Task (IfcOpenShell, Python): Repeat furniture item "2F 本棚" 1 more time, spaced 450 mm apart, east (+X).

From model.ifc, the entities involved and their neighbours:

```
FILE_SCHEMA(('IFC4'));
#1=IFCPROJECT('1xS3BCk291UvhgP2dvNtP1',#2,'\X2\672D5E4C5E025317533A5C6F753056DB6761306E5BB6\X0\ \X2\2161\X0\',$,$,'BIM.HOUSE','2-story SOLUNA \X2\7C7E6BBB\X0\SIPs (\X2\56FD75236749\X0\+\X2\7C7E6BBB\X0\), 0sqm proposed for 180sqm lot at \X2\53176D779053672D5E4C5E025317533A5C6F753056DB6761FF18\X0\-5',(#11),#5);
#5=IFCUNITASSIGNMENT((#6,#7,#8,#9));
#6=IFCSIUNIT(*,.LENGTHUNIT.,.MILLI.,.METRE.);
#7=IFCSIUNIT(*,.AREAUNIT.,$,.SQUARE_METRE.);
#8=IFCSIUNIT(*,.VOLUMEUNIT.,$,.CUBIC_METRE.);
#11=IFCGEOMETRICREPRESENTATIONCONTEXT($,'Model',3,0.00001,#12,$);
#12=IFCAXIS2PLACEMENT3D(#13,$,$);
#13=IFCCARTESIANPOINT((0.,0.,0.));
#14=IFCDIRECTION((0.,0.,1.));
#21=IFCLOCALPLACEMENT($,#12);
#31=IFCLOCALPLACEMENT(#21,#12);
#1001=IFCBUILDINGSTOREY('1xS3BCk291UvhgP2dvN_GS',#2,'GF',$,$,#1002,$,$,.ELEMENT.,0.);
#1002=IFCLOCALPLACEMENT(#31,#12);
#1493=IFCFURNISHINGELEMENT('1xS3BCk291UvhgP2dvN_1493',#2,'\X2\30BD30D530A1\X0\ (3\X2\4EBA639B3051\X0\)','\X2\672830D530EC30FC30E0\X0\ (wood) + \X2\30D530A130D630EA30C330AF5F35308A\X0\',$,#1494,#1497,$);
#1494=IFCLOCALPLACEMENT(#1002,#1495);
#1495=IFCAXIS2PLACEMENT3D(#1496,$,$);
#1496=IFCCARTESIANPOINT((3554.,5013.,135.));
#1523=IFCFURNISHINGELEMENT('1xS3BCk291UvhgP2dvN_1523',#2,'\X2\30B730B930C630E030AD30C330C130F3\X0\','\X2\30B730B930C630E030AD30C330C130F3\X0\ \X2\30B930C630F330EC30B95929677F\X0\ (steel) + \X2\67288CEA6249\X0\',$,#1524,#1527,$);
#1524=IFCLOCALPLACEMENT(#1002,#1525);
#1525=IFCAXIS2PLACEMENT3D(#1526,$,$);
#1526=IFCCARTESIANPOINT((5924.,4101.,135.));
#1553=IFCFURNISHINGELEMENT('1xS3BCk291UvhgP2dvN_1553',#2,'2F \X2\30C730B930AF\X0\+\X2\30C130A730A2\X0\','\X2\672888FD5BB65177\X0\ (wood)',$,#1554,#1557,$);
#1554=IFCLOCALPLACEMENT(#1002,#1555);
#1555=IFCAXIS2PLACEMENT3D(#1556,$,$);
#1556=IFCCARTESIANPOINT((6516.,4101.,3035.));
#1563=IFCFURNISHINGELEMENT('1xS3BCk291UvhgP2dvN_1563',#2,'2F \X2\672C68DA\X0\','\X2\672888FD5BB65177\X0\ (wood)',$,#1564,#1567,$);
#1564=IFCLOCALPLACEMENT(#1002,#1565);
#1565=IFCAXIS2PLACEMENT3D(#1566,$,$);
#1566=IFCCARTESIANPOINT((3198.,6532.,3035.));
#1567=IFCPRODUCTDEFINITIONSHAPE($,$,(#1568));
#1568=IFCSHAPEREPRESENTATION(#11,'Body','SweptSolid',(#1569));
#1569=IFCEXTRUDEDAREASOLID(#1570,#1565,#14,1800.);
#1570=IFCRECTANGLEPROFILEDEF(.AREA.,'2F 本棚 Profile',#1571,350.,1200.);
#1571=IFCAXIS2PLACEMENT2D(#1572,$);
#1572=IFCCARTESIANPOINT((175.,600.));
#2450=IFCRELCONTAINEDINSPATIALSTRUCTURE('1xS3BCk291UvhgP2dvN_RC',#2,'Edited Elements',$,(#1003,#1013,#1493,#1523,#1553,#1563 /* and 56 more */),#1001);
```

```python
import numpy as np
import ifcopenshell
import ifcopenshell.api.geometry
import ifcopenshell.api.root
import ifcopenshell.util.element
import ifcopenshell.util.placement

model = ifcopenshell.open("model.ifc")


def reuse_history(source, copy):
    """copy_class also copies each property set's owner history, people and application; keep the originals."""
    for rel in copy.IsDefinedBy:
        if rel.is_a("IfcRelDefinesByProperties") and (history := rel.RelatingPropertyDefinition.OwnerHistory):
            rel.RelatingPropertyDefinition.OwnerHistory = source.OwnerHistory
            ifcopenshell.util.element.remove_deep2(model, history)


source = model.by_id(1563)
base = ifcopenshell.util.placement.get_local_placement(source.ObjectPlacement)
step = np.array([1.0, 0.0, 0.0]) * 450.0

for i in range(1, 2):
    copy = ifcopenshell.api.root.copy_class(model, product=source)
    copy.Representation = ifcopenshell.util.element.copy_deep(
        model, source.Representation, exclude=["IfcGeometricRepresentationContext", "IfcRepresentationMap"]
    )
    reuse_history(source, copy)
    matrix = base.copy()
    matrix[:3, 3] += i * step
    print("added at", matrix[:3, 3].round(3) + 0.0)
    ifcopenshell.api.geometry.edit_object_placement(model, product=copy, matrix=matrix, is_si=False)

model.write("model_updated.ifc")
```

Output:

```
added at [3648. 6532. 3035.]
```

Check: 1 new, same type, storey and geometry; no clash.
